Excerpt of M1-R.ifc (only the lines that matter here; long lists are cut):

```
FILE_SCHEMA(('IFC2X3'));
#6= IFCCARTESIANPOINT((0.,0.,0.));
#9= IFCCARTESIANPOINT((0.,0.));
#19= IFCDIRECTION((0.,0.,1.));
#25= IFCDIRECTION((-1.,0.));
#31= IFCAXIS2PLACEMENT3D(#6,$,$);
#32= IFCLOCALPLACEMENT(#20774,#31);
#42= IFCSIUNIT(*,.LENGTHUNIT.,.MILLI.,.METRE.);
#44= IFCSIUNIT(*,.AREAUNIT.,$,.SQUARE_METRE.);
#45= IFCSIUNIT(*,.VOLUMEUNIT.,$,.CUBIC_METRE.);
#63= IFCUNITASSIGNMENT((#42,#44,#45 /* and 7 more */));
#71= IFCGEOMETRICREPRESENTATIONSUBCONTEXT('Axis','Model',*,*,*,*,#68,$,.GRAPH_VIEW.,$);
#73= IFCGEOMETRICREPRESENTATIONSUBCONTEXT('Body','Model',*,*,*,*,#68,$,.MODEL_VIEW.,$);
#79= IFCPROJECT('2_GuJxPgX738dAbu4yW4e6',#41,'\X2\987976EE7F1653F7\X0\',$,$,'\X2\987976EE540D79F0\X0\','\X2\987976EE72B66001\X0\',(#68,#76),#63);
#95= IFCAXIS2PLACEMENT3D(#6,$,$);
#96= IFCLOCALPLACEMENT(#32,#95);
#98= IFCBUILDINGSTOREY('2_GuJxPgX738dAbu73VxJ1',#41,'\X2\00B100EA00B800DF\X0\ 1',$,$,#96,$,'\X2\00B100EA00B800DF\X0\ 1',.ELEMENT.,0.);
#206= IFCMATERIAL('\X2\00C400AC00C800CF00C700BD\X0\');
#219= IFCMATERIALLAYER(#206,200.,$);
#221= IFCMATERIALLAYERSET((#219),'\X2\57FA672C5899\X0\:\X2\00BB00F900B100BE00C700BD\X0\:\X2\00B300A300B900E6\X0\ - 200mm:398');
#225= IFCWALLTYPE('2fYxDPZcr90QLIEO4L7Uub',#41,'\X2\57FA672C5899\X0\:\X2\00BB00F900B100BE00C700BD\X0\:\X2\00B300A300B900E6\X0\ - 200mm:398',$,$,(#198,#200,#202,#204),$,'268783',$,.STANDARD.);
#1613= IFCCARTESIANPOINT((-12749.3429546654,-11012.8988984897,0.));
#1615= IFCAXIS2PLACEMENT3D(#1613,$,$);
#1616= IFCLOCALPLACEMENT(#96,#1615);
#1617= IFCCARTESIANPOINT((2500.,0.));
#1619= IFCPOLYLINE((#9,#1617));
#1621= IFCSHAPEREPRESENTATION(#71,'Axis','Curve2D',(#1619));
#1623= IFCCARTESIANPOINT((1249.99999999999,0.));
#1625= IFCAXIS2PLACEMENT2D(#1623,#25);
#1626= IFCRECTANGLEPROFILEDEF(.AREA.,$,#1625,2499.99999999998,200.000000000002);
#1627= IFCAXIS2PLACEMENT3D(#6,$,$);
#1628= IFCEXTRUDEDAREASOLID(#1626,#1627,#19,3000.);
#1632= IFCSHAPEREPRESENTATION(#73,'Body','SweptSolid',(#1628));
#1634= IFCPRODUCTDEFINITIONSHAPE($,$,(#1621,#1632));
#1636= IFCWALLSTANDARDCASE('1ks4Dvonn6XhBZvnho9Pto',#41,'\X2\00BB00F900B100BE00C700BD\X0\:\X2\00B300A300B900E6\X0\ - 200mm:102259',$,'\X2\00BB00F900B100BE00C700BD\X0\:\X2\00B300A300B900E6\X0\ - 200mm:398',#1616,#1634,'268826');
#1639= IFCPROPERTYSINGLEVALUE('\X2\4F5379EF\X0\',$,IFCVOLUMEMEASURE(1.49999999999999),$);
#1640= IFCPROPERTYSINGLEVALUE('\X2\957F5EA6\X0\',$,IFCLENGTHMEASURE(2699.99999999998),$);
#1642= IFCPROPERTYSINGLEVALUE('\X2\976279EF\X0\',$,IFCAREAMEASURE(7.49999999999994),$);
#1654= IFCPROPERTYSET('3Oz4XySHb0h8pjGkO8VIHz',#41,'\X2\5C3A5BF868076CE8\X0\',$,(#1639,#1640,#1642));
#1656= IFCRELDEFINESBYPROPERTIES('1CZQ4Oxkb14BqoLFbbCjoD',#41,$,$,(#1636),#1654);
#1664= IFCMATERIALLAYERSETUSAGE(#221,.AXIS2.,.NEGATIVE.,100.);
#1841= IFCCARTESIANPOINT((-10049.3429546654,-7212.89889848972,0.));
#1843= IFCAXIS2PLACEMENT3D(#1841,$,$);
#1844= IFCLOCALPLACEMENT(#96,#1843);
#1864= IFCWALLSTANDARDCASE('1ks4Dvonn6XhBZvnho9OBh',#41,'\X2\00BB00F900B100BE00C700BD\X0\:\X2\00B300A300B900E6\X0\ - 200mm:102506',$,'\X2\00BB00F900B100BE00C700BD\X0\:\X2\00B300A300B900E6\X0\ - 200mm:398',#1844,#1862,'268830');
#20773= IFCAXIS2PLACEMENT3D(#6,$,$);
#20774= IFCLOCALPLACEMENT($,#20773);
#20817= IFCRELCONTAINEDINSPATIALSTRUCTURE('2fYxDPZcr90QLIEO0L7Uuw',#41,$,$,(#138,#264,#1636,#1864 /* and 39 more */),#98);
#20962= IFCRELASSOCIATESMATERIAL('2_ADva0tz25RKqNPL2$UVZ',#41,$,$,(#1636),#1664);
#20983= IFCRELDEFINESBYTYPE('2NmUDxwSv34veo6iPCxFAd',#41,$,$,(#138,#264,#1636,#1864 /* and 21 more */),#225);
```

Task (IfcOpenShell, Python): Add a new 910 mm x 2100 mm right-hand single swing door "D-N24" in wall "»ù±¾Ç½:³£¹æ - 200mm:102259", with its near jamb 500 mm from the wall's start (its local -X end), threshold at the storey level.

```python
import numpy as np
import ifcopenshell
import ifcopenshell.api.feature
import ifcopenshell.api.geometry
import ifcopenshell.api.pset
import ifcopenshell.api.root
import ifcopenshell.api.spatial
import ifcopenshell.api.type
import ifcopenshell.geom
import ifcopenshell.util.element
import ifcopenshell.util.placement
import ifcopenshell.util.representation
import ifcopenshell.util.shape
import ifcopenshell.util.unit

model = ifcopenshell.open("M1-R.ifc")
unit_scale = ifcopenshell.util.unit.calculate_unit_scale(model)
area_scale = ifcopenshell.util.unit.calculate_unit_scale(model, "AREAUNIT")
volume_scale = ifcopenshell.util.unit.calculate_unit_scale(model, "VOLUMEUNIT")
settings = ifcopenshell.geom.settings()


def volume(element):
    """Net volume in cubic metres, openings subtracted."""
    shape = ifcopenshell.geom.create_shape(settings, element)
    return ifcopenshell.util.shape.get_volume(shape.geometry)


wall = model.by_guid("1ks4Dvonn6XhBZvnho9Pto")
storey = ifcopenshell.util.element.get_container(wall, ifc_class="IfcBuildingStorey")
context = ifcopenshell.util.representation.get_context(model, "Model", "Body", "MODEL_VIEW")
before = volume(wall)

width, height, from_end, sill = 0.91, 2.1, 0.5, 0.0  # metres

# The wall runs along its own X axis, and the end named is its -X end.
wall_shape = ifcopenshell.geom.create_shape(settings, wall)
x, y, z = ifcopenshell.util.shape.get_vertices(wall_shape.geometry).T
start = x.min() + from_end
face, thickness = float(y.min()), float(y.max() - y.min())
wall_matrix = ifcopenshell.util.placement.get_local_placement(wall.ObjectPlacement)
level = ifcopenshell.util.placement.get_local_placement(storey.ObjectPlacement)[2, 3]


def in_wall(x, y):
    """Placement at x, y metres in the wall's axes, at sill height."""
    matrix = wall_matrix.copy()
    matrix[:, 3] = wall_matrix @ np.array([x / unit_scale, y / unit_scale, 0.0, 1.0])
    matrix[2, 3] = level + sill / unit_scale
    return matrix


# Opening: a box that overshoots both wall faces by 50 mm.
opening = ifcopenshell.api.root.create_entity(model, ifc_class="IfcOpeningElement")
box = ifcopenshell.api.geometry.add_wall_representation(
    model, context=context, length=width, height=height, thickness=thickness + 0.1
)
ifcopenshell.api.geometry.assign_representation(model, product=opening, representation=box)
ifcopenshell.api.geometry.edit_object_placement(model, product=opening, matrix=in_wall(start, face - 0.05), is_si=False)
ifcopenshell.api.feature.add_feature(model, feature=opening, element=wall)

door = ifcopenshell.api.root.create_entity(model, ifc_class="IfcDoor", name="D-N24")
door.OverallWidth, door.OverallHeight = width / unit_scale, height / unit_scale
body = ifcopenshell.api.geometry.add_door_representation(
    model,
    context=context,
    overall_width=door.OverallWidth,
    overall_height=door.OverallHeight,
    operation_type="SINGLE_SWING_RIGHT",
    lining_properties={"LiningDepth": thickness / unit_scale, "ThresholdDepth": thickness / unit_scale},
)
ifcopenshell.api.geometry.assign_representation(model, product=door, representation=body)
ifcopenshell.api.spatial.assign_container(model, products=[door], relating_structure=storey)
fills = ifcopenshell.api.feature.add_filling(model, opening=opening, element=door)
fills.OwnerHistory = door.OwnerHistory  # required in IFC2X3

# IFC2X3 keeps the operation on the door style.
style = ifcopenshell.api.root.create_entity(model, ifc_class="IfcDoorStyle", name="D-N24")
style.OperationType, style.ConstructionType = "SINGLE_SWING_RIGHT", "NOTDEFINED"
style.ParameterTakesPrecedence = style.Sizeable = False
ifcopenshell.api.type.assign_type(model, related_objects=[door], relating_type=style)

# The lining spans the wall, so the door starts at the wall face.
ifcopenshell.api.geometry.edit_object_placement(model, product=door, matrix=in_wall(start, face), is_si=False)

after = volume(wall)

# Update the wall's stored quantities.
pset = model.by_id(ifcopenshell.util.element.get_pset(wall, "尺寸标注", should_inherit=False)["id"])
ifcopenshell.api.pset.edit_pset(model, pset=pset, properties={
    "体积": model.create_entity("IfcVolumeMeasure", after / volume_scale),
    "面积": model.create_entity("IfcAreaMeasure", after / thickness / area_scale),
})

print(f"wall volume {before:.3f} -> {after:.3f} m3")

model.write("M1-R_edited.ifc")
```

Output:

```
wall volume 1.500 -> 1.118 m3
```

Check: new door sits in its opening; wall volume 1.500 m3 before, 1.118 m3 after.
